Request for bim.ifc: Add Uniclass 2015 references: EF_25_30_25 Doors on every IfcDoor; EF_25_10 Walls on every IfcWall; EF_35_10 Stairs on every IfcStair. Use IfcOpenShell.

First a look at what the model holds.

```python
import ifcopenshell

model = ifcopenshell.open("bim.ifc")
print(model.schema)
print("classifications:", [c.Name for c in model.by_type("IfcClassification")])
for ifc_class in ("IfcDoor", "IfcRoof", "IfcStair", "IfcWall", "IfcWindow"):
    print(ifc_class, len(model.by_type(ifc_class)))
```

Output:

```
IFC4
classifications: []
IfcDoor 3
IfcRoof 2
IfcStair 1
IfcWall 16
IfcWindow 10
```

```python
import ifcopenshell
import ifcopenshell.api.classification

model = ifcopenshell.open("bim.ifc")

system = ifcopenshell.api.classification.add_classification(model, classification="Uniclass 2015")

codes = {
    "IfcDoor": ("EF_25_30_25", "Doors"),
    "IfcWall": ("EF_25_10", "Walls"),
    "IfcStair": ("EF_35_10", "Stairs"),
}
for ifc_class, (code, name) in codes.items():
    products = model.by_type(ifc_class)
    ifcopenshell.api.classification.add_reference(
        model, products=products, classification=system, identification=code, name=name
    )
    print(code, len(products))

model.write("bim_updated.ifc")
```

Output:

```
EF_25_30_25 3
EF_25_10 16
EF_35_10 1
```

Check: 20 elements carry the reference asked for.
